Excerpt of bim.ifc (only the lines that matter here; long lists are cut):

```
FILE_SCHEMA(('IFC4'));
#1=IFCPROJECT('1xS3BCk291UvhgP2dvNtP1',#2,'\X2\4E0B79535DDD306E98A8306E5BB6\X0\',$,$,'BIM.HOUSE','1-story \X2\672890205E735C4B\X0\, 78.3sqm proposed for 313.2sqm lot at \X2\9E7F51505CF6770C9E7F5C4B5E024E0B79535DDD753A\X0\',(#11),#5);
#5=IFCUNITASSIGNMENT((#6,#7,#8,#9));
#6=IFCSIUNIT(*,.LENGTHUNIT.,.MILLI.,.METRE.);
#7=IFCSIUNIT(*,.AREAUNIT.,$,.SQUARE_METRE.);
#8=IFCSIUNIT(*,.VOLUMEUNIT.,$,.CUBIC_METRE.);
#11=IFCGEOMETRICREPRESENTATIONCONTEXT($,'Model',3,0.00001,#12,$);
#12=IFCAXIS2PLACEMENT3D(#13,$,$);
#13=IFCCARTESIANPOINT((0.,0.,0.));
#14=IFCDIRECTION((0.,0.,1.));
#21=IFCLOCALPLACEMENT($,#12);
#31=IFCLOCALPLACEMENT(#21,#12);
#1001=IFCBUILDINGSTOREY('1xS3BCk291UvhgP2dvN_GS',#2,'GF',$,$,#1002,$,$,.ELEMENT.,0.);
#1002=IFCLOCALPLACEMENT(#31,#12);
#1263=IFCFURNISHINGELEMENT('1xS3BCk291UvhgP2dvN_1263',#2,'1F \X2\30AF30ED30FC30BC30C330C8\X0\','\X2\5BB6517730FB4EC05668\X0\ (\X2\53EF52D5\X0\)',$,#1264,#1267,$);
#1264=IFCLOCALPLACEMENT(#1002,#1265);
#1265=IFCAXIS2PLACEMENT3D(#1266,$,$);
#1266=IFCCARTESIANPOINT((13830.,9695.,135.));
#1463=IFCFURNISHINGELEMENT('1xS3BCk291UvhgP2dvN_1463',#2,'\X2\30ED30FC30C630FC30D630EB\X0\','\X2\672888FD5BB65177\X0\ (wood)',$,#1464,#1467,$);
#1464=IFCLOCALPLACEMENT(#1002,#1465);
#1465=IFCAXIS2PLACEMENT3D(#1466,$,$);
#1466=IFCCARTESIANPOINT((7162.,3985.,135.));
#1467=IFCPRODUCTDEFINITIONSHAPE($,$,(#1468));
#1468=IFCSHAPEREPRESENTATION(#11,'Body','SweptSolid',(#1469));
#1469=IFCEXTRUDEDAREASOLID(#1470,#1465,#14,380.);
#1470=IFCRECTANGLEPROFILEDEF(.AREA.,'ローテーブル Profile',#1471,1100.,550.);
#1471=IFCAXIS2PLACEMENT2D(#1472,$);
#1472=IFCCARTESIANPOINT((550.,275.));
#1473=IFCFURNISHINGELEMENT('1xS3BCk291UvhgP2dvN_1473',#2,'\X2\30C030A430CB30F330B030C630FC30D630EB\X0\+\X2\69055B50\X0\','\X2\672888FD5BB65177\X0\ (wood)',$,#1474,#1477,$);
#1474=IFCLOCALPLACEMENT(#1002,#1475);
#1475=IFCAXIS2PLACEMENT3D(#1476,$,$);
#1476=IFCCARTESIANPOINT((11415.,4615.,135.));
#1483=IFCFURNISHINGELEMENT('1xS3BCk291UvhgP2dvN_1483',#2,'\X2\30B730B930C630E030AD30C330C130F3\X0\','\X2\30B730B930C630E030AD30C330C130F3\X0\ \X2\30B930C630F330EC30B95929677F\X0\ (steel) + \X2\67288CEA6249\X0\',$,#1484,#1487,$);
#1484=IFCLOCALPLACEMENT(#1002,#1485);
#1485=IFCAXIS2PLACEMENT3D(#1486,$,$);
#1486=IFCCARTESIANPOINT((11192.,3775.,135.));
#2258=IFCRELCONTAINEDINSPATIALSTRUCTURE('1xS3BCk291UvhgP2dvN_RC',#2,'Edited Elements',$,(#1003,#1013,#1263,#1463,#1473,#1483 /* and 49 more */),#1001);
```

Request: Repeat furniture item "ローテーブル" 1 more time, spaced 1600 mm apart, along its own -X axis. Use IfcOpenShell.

```python
import ifcopenshell
import ifcopenshell.api.geometry
import ifcopenshell.api.root
import ifcopenshell.util.element
import ifcopenshell.util.placement

model = ifcopenshell.open("bim.ifc")


def reuse_history(source, copy):
    """copy_class also copies each property set's owner history, people and application; keep the originals."""
    for rel in copy.IsDefinedBy:
        if rel.is_a("IfcRelDefinesByProperties") and (history := rel.RelatingPropertyDefinition.OwnerHistory):
            rel.RelatingPropertyDefinition.OwnerHistory = source.OwnerHistory
            ifcopenshell.util.element.remove_deep2(model, history)


source = model.by_guid("1xS3BCk291UvhgP2dvN_1463")
base = ifcopenshell.util.placement.get_local_placement(source.ObjectPlacement)
step = -base[:3, 0] * 1600.0

for i in range(1, 2):
    copy = ifcopenshell.api.root.copy_class(model, product=source)
    copy.Representation = ifcopenshell.util.element.copy_deep(
        model, source.Representation, exclude=["IfcGeometricRepresentationContext", "IfcRepresentationMap"]
    )
    reuse_history(source, copy)
    matrix = base.copy()
    matrix[:3, 3] += i * step
    print("added at", matrix[:3, 3].round(3) + 0.0)
    ifcopenshell.api.geometry.edit_object_placement(model, product=copy, matrix=matrix, is_si=False)

model.write("bim_rev.ifc")
```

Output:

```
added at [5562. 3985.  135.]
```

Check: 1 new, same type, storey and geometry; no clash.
